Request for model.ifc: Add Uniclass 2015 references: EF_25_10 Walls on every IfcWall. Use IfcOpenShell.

First a look at what the model holds.

```python
import ifcopenshell

model = ifcopenshell.open("model.ifc")
print(model.schema)
print("classifications:", [c.Name for c in model.by_type("IfcClassification")])
for ifc_class in ("IfcDoor", "IfcRoof", "IfcStair", "IfcWall", "IfcWindow"):
    print(ifc_class, len(model.by_type(ifc_class)))
```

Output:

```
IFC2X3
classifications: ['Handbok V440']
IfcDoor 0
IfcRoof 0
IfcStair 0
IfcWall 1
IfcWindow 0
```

```python
import ifcopenshell
import ifcopenshell.api.classification

model = ifcopenshell.open("model.ifc")

# IFC2X3 requires Source and Edition and has no link from the project to the system.
system = model.create_entity("IfcClassification", Source="NBS", Edition="2015", Name="Uniclass 2015")

codes = {
    "IfcWall": ("EF_25_10", "Walls"),
}
for ifc_class, (code, name) in codes.items():
    products = model.by_type(ifc_class)
    ifcopenshell.api.classification.add_reference(
        model, products=products, classification=system, identification=code, name=name
    )
    print(code, len(products))

model.write("model-out.ifc")
```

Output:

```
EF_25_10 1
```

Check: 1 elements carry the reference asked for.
